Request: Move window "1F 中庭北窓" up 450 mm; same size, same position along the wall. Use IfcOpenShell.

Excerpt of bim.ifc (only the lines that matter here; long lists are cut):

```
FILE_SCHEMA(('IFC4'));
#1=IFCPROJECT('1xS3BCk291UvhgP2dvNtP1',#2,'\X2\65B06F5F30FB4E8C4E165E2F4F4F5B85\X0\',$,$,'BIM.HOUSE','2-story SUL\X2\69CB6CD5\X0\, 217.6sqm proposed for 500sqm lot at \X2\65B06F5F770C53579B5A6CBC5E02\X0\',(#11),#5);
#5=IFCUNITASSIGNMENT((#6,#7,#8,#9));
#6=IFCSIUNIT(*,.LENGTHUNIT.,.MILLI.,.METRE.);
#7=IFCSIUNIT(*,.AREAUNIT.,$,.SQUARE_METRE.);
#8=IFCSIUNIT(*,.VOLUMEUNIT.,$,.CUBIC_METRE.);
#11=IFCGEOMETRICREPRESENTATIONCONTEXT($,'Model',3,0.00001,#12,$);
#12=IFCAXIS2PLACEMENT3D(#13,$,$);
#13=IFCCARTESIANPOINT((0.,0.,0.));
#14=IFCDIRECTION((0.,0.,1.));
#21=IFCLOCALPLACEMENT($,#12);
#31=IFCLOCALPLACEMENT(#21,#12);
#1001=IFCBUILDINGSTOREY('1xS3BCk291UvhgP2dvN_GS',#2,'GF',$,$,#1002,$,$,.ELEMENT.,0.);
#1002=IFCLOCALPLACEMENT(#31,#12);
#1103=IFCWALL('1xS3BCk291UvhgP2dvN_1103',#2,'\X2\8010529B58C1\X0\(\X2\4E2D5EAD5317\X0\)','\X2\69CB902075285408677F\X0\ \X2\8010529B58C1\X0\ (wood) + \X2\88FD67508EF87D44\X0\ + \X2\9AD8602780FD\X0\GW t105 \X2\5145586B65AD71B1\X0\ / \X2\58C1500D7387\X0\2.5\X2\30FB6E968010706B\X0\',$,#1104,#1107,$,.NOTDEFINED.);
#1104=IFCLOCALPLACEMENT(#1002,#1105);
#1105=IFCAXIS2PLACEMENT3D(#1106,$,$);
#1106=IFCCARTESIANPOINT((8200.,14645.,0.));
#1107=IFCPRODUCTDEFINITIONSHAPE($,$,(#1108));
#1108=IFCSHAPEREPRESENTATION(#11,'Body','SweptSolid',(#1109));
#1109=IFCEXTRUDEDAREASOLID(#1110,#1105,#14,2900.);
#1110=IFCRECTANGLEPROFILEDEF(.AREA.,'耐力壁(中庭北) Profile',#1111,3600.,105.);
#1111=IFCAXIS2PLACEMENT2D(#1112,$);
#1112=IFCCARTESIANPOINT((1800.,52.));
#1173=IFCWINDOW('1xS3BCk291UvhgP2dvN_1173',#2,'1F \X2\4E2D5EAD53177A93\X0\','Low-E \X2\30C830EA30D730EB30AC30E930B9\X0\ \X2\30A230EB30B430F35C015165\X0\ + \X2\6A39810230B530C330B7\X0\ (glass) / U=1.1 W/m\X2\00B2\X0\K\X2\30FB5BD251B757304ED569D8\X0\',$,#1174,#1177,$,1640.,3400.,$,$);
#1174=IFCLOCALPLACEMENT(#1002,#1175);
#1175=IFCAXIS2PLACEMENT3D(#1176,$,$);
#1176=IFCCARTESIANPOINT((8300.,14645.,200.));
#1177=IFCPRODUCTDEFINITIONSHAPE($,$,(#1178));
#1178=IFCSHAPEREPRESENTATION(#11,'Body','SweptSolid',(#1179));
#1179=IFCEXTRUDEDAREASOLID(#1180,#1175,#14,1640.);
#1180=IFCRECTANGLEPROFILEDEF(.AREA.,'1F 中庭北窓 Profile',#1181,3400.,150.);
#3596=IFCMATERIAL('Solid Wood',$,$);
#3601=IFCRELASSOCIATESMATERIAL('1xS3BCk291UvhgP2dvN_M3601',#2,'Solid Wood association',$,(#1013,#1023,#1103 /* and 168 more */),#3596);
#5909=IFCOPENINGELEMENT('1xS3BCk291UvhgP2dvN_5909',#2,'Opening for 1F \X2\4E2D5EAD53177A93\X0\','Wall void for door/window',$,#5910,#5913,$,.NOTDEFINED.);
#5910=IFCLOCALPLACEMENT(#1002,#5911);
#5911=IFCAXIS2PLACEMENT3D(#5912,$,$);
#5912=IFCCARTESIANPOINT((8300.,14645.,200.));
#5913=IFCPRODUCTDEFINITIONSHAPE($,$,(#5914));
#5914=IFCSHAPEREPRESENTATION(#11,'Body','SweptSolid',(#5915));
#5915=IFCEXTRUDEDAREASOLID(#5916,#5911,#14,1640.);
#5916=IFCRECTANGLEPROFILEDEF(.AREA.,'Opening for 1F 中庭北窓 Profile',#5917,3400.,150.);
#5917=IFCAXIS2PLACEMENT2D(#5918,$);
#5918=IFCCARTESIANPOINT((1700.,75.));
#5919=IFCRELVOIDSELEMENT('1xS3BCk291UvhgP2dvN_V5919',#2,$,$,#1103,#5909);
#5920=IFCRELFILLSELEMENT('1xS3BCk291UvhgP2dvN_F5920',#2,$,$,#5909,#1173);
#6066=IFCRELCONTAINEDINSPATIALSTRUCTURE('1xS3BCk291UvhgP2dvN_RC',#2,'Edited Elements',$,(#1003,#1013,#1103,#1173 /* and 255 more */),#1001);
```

```python
import numpy as np
import ifcopenshell
import ifcopenshell.api.geometry
import ifcopenshell.util.placement
import ifcopenshell.util.unit

model = ifcopenshell.open("bim.ifc")
unit_scale = ifcopenshell.util.unit.calculate_unit_scale(model)

window = model.by_id(1173)
opening = window.FillsVoids[0].RelatingOpeningElement
dz = 450.0

shift = np.array([0.0, 0.0, dz])
# The window is not placed relative to its opening, so move both.
for product in (opening, window):
    matrix = ifcopenshell.util.placement.get_local_placement(product.ObjectPlacement)
    matrix[:3, 3] += shift
    ifcopenshell.api.geometry.edit_object_placement(model, product=product, matrix=matrix, is_si=False)

print(f"moved by {dz * unit_scale:+.3f} m")

model.write("bim_rev.ifc")
```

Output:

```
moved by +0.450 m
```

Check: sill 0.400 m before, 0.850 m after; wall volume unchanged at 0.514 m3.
